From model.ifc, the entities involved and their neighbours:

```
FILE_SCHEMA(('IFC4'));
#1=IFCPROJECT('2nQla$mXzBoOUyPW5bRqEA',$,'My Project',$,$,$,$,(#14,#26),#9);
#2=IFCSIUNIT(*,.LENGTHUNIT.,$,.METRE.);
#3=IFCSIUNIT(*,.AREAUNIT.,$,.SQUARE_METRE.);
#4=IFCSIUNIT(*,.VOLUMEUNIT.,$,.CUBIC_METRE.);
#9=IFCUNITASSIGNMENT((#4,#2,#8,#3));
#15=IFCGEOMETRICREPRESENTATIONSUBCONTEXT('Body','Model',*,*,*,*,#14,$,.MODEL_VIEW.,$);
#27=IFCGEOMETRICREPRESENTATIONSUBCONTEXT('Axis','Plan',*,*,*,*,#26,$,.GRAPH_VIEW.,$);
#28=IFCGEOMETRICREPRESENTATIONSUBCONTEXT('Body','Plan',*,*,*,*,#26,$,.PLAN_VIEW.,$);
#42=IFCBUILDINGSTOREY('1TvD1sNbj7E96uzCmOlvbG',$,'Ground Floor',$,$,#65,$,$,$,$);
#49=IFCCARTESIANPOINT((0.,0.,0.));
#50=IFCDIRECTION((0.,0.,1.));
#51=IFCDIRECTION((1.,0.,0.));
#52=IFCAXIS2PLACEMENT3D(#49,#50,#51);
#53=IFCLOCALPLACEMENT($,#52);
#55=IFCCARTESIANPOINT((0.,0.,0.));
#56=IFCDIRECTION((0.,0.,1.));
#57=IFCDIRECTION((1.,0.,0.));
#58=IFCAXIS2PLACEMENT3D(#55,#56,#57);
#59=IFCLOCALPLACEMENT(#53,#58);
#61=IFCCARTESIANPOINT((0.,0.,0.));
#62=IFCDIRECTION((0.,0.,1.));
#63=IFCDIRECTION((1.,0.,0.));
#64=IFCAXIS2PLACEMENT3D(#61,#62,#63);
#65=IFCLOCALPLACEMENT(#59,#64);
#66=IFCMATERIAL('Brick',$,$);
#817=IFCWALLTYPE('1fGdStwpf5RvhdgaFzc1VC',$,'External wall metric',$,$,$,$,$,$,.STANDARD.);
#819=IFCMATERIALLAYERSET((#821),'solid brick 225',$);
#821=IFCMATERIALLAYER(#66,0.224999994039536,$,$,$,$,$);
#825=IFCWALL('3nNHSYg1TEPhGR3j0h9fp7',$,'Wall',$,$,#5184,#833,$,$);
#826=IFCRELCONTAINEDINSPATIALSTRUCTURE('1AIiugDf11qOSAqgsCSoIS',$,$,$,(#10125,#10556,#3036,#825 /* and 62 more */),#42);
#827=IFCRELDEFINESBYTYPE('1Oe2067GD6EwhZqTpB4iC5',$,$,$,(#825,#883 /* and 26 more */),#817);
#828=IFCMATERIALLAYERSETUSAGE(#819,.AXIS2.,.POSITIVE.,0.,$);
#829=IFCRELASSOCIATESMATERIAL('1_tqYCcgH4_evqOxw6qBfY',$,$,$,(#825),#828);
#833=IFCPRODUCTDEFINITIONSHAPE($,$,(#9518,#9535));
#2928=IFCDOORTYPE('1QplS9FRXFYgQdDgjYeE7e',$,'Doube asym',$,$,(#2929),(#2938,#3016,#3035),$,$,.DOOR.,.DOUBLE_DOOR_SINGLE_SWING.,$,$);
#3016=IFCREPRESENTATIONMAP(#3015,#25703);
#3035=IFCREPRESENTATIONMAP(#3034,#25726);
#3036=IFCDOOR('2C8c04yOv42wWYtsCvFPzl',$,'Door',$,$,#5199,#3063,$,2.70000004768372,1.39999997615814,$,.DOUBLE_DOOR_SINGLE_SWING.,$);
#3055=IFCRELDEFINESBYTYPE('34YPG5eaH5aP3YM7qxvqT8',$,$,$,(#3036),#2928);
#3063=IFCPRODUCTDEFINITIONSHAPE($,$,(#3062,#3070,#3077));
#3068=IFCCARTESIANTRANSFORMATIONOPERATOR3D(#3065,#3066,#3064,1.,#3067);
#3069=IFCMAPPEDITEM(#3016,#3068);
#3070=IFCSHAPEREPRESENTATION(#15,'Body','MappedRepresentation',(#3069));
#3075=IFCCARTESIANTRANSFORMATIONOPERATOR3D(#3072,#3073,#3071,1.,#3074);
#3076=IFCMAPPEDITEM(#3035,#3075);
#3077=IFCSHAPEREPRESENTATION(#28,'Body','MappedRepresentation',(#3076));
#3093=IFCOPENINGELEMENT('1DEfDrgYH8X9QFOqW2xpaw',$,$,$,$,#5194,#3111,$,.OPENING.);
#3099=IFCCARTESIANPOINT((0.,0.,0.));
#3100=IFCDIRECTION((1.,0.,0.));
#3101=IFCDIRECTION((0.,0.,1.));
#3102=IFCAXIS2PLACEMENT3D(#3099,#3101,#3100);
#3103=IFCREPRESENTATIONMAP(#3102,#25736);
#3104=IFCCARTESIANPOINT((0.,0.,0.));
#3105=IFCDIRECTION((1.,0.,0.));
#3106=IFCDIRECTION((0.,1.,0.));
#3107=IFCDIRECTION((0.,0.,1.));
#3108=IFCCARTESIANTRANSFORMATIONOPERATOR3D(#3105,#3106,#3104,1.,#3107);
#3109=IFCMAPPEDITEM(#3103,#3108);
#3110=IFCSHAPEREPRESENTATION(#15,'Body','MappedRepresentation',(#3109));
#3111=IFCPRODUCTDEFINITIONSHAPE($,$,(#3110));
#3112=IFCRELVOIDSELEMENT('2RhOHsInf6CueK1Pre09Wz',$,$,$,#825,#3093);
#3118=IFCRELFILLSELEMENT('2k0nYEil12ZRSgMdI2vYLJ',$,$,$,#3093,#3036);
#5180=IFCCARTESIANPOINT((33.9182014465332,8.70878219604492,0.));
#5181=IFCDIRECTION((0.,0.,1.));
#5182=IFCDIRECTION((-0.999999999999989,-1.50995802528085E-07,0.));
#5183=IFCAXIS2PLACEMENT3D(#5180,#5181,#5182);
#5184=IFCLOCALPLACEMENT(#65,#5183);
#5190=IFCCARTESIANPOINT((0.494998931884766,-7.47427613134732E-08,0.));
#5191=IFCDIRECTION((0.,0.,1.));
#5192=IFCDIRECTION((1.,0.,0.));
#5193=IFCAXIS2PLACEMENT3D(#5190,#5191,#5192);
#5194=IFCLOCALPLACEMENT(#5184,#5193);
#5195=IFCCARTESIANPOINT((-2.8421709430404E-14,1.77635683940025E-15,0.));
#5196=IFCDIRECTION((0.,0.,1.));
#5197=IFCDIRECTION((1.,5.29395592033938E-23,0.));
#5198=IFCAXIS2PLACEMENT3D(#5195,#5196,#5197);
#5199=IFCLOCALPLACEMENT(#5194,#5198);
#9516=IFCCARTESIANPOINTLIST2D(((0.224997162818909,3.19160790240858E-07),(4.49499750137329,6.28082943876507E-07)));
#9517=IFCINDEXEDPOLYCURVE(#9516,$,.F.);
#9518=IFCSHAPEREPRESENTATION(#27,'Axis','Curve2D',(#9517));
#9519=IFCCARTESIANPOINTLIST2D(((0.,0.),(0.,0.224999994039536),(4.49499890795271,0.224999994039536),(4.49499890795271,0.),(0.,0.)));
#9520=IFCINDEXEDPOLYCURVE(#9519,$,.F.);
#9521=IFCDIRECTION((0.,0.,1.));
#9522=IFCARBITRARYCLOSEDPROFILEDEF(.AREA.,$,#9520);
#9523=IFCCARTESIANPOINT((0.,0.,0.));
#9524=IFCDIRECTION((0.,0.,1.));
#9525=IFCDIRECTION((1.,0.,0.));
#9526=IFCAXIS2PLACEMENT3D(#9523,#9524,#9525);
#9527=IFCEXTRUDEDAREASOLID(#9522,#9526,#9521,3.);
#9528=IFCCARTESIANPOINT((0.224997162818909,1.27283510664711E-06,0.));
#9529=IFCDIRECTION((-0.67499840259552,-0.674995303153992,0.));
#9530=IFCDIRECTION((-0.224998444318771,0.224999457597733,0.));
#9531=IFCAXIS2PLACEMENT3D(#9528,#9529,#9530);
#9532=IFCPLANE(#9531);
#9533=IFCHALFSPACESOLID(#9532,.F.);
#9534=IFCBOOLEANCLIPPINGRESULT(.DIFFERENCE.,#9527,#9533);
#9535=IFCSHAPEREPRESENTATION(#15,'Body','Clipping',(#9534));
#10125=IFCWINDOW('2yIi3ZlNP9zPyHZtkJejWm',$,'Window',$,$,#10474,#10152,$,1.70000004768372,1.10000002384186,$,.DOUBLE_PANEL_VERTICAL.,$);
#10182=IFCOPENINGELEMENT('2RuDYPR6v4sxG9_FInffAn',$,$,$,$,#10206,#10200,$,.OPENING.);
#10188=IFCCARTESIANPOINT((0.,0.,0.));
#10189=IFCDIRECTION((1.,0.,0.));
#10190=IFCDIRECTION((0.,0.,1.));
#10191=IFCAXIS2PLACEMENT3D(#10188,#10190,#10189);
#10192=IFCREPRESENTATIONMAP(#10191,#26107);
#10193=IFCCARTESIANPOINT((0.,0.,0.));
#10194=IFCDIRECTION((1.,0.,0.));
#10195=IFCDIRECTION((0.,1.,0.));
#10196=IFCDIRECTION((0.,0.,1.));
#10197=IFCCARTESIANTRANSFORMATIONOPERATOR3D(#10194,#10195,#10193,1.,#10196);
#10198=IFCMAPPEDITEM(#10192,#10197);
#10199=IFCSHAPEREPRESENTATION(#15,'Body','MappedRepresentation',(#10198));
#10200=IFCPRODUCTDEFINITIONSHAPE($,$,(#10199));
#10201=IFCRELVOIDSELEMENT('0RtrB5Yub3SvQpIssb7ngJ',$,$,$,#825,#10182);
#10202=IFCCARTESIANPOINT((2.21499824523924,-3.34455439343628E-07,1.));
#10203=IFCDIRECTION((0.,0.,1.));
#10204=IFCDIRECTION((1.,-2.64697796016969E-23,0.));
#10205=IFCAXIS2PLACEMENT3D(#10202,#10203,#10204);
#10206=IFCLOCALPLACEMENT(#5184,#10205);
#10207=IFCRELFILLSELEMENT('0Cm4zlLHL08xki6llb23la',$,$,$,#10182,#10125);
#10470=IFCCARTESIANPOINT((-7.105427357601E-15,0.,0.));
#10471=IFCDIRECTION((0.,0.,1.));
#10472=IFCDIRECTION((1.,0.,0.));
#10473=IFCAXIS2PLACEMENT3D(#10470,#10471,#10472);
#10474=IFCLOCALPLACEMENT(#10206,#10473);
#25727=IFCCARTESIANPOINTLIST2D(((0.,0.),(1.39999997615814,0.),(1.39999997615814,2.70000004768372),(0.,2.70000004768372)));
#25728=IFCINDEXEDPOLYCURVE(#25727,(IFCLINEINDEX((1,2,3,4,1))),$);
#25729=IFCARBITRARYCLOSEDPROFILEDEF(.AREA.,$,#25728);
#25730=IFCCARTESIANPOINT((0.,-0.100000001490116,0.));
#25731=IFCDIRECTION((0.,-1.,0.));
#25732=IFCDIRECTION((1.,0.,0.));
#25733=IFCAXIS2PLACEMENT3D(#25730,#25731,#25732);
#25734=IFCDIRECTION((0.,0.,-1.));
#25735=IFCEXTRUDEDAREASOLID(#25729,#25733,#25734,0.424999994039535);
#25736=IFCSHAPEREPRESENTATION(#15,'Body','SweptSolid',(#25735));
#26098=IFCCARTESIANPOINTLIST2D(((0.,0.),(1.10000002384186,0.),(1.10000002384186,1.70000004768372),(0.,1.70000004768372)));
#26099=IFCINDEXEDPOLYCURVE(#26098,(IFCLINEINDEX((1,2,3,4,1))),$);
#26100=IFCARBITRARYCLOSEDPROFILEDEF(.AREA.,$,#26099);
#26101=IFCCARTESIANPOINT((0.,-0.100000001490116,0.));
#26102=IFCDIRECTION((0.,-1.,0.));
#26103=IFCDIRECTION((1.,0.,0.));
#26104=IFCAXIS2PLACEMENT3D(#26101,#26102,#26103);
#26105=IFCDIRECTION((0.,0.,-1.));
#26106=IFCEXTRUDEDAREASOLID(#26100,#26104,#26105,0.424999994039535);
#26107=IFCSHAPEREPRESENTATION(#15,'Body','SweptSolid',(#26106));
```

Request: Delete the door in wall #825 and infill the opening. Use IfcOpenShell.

```python
import ifcopenshell
import ifcopenshell.api.feature
import ifcopenshell.api.root
import ifcopenshell.geom
import ifcopenshell.util.shape

model = ifcopenshell.open("model.ifc")
settings = ifcopenshell.geom.settings()


def volume(element):
    """Net volume in cubic metres, openings subtracted."""
    shape = ifcopenshell.geom.create_shape(settings, element)
    return ifcopenshell.util.shape.get_volume(shape.geometry)


door = model.by_id(3036)
opening = door.FillsVoids[0].RelatingOpeningElement
wall = opening.VoidsElements[0].RelatingBuildingElement
before = volume(wall)

ifcopenshell.api.root.remove_product(model, product=door)
ifcopenshell.api.feature.remove_feature(model, feature=opening)

after = volume(wall)

print(f"wall volume {before:.3f} -> {after:.3f} m3")

model.write("model_updated.ifc")
```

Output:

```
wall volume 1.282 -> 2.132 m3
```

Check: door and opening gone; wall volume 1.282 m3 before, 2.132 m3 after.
